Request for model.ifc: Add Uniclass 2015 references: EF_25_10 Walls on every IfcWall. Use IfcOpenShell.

First a look at what the model holds.

```python
import ifcopenshell

model = ifcopenshell.open("model.ifc")
print(model.schema)
print("classifications:", [c.Name for c in model.by_type("IfcClassification")])
for ifc_class in ("IfcDoor", "IfcRoof", "IfcStair", "IfcWall", "IfcWindow"):
    print(ifc_class, len(model.by_type(ifc_class)))
```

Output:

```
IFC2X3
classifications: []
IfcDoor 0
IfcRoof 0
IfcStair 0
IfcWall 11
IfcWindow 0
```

```python
import ifcopenshell
import ifcopenshell.api.classification

model = ifcopenshell.open("model.ifc")

# IFC2X3 requires Source and Edition and has no link from the project to the system.
system = model.create_entity("IfcClassification", Source="NBS", Edition="2015", Name="Uniclass 2015")

codes = {
    "IfcWall": ("EF_25_10", "Walls"),
}
for ifc_class, (code, name) in codes.items():
    products = model.by_type(ifc_class)
    ifcopenshell.api.classification.add_reference(
        model, products=products, classification=system, identification=code, name=name
    )
    print(code, len(products))

model.write("model_edited.ifc")
```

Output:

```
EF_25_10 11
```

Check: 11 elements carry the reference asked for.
